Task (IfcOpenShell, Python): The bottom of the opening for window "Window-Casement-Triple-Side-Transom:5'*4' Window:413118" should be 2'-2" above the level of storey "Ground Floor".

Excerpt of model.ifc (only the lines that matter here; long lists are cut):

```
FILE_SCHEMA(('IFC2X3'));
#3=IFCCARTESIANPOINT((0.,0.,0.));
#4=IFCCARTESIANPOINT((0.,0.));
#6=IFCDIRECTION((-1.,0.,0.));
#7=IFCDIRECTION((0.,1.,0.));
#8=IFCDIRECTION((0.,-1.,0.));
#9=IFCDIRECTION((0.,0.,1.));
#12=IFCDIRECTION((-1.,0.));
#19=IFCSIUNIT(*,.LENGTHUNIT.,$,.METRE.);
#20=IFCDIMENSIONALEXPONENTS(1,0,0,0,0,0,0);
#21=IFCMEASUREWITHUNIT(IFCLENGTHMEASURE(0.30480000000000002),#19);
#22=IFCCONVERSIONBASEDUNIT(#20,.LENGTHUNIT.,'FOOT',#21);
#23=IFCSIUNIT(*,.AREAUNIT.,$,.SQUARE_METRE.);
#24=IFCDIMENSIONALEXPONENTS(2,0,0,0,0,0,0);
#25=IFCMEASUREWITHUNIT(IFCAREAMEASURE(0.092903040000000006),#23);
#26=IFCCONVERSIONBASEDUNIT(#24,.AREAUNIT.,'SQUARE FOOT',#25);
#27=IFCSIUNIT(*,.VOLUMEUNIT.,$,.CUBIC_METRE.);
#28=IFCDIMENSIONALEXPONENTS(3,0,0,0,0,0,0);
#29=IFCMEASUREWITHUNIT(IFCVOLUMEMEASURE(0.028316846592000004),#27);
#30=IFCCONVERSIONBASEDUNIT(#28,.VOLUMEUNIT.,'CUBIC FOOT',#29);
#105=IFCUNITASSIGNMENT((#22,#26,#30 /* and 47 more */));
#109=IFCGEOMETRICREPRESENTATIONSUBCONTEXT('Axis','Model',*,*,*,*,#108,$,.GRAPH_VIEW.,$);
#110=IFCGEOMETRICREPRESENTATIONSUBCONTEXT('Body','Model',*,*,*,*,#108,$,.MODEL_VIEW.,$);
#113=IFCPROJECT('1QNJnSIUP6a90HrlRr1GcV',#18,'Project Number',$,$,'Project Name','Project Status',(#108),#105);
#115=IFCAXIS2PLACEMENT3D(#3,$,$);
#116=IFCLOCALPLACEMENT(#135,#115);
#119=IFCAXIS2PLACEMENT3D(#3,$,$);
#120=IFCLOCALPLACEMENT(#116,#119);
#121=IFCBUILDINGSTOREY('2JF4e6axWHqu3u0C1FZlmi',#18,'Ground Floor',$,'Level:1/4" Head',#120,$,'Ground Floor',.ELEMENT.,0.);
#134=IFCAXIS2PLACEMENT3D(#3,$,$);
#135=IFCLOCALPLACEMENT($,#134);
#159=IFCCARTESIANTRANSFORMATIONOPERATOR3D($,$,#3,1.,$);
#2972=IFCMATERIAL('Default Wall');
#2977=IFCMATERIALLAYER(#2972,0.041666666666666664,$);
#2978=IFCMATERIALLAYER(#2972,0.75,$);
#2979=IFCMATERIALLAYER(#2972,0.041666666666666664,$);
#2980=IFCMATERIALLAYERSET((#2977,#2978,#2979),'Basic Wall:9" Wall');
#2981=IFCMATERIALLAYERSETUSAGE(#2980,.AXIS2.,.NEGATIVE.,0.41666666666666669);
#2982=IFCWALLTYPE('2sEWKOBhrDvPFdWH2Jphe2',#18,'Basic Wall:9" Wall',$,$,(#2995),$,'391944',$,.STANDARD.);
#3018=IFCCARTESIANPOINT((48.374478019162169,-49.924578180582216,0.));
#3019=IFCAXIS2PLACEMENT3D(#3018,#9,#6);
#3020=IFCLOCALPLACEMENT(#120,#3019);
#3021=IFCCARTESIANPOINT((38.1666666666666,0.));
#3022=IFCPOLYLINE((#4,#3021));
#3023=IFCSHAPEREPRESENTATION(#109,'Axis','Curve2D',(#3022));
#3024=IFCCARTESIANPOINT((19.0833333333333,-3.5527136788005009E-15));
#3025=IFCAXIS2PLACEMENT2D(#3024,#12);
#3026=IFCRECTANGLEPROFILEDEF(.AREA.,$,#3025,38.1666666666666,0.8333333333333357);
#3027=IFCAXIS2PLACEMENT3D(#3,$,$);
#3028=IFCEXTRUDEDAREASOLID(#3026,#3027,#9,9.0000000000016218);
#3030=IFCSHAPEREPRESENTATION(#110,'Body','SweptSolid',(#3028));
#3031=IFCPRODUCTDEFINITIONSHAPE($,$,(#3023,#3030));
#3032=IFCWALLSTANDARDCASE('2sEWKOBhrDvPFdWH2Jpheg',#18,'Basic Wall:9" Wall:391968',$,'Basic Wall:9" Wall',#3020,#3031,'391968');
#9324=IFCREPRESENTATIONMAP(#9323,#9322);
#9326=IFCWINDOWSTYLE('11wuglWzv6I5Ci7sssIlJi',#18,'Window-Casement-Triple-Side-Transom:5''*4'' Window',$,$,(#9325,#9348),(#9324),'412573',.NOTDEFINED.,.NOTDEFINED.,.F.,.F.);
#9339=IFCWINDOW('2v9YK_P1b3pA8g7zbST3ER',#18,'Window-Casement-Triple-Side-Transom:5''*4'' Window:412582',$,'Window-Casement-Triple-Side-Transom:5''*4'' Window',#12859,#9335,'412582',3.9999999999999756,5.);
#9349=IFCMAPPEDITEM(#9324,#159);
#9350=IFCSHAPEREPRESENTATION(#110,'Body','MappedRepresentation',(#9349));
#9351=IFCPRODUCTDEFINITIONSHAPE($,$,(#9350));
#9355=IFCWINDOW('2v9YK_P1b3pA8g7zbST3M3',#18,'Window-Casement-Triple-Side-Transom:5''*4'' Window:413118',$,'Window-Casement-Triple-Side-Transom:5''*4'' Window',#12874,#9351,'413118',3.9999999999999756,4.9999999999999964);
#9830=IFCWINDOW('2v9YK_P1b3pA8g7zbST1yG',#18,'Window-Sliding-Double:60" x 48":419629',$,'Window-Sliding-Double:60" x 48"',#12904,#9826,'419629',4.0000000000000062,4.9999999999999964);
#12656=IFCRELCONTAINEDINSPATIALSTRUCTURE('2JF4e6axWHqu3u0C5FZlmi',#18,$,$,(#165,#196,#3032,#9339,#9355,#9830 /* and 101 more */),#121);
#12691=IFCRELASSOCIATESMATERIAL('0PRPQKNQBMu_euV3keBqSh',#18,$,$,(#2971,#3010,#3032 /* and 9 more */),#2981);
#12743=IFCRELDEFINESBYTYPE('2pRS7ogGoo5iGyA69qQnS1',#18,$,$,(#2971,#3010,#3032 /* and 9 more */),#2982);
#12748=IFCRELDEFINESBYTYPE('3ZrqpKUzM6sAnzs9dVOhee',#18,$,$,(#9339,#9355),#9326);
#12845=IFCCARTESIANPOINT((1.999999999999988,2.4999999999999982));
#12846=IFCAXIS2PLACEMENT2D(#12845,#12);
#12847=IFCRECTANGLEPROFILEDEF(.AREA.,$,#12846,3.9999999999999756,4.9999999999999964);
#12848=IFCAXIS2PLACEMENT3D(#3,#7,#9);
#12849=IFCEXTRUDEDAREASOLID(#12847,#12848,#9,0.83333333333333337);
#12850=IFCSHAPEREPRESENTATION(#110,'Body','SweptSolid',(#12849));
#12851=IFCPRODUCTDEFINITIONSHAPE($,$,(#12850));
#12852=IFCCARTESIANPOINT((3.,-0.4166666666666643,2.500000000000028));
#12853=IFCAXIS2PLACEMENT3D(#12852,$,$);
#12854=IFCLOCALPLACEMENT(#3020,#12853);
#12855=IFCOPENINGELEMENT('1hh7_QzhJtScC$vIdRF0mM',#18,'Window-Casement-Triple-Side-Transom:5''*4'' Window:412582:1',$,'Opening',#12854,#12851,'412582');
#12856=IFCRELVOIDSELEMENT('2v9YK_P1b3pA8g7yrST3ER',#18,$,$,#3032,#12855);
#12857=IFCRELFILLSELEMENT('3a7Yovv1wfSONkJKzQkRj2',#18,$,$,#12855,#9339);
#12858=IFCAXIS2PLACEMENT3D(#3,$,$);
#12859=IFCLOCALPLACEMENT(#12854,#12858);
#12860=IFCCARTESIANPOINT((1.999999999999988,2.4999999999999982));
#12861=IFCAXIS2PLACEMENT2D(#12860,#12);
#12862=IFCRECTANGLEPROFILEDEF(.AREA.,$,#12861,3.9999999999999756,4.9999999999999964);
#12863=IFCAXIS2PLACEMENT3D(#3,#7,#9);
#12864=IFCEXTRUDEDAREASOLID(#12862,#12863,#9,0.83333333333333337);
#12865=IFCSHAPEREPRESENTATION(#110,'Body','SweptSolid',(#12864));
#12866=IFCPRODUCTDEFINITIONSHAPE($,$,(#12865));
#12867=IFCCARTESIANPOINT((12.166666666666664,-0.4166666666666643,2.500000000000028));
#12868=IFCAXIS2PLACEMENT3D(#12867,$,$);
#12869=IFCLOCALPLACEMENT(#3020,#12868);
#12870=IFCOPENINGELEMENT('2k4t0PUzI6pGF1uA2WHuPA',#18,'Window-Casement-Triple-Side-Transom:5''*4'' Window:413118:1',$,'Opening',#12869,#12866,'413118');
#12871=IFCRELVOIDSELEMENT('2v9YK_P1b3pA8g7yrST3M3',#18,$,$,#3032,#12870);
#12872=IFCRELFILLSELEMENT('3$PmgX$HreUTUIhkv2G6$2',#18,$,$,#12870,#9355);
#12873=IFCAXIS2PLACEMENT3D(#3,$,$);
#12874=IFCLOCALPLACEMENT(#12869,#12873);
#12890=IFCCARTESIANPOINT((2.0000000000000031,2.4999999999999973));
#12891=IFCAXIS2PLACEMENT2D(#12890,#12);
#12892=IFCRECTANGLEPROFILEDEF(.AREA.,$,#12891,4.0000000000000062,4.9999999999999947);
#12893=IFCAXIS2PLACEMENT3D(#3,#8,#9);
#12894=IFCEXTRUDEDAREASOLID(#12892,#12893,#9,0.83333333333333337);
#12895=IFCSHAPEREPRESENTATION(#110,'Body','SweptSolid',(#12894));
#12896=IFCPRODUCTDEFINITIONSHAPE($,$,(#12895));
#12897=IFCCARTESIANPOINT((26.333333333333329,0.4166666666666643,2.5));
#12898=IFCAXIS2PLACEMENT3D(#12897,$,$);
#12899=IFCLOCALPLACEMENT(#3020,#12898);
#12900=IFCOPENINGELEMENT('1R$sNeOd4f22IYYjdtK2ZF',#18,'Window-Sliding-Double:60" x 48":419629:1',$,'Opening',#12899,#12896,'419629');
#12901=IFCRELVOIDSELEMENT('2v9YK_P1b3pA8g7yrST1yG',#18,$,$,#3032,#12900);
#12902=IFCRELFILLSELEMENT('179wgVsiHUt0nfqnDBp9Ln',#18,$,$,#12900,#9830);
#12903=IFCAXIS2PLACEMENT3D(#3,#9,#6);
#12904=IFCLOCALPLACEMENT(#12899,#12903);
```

```python
import numpy as np
import ifcopenshell
import ifcopenshell.api.geometry
import ifcopenshell.geom
import ifcopenshell.util.element
import ifcopenshell.util.placement
import ifcopenshell.util.shape
import ifcopenshell.util.unit

model = ifcopenshell.open("model.ifc")
unit_scale = ifcopenshell.util.unit.calculate_unit_scale(model)

window = model.by_id(9355)
opening = window.FillsVoids[0].RelatingOpeningElement
storey = ifcopenshell.util.element.get_container(window, ifc_class="IfcBuildingStorey")
level = ifcopenshell.util.placement.get_local_placement(storey.ObjectPlacement)[2, 3]

# The opening's origin need not be at the sill, so measure its lowest point.
shape = ifcopenshell.geom.create_shape(ifcopenshell.geom.settings(), opening)
bottom = ifcopenshell.util.shape.get_shape_bottom_elevation(shape, shape.geometry) / unit_scale
dz = level + 26 * 0.0254 / unit_scale - bottom

shift = np.array([0.0, 0.0, dz])
# The window is placed relative to its opening, so it follows when the opening moves.
matrix = ifcopenshell.util.placement.get_local_placement(opening.ObjectPlacement)
matrix[:3, 3] += shift
ifcopenshell.api.geometry.edit_object_placement(
    model, product=opening, matrix=matrix, is_si=False, should_transform_children=True
)

print(f"moved by {dz * unit_scale:+.3f} m")

model.write("model_rev.ifc")
```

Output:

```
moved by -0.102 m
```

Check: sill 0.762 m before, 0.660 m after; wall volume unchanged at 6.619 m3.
